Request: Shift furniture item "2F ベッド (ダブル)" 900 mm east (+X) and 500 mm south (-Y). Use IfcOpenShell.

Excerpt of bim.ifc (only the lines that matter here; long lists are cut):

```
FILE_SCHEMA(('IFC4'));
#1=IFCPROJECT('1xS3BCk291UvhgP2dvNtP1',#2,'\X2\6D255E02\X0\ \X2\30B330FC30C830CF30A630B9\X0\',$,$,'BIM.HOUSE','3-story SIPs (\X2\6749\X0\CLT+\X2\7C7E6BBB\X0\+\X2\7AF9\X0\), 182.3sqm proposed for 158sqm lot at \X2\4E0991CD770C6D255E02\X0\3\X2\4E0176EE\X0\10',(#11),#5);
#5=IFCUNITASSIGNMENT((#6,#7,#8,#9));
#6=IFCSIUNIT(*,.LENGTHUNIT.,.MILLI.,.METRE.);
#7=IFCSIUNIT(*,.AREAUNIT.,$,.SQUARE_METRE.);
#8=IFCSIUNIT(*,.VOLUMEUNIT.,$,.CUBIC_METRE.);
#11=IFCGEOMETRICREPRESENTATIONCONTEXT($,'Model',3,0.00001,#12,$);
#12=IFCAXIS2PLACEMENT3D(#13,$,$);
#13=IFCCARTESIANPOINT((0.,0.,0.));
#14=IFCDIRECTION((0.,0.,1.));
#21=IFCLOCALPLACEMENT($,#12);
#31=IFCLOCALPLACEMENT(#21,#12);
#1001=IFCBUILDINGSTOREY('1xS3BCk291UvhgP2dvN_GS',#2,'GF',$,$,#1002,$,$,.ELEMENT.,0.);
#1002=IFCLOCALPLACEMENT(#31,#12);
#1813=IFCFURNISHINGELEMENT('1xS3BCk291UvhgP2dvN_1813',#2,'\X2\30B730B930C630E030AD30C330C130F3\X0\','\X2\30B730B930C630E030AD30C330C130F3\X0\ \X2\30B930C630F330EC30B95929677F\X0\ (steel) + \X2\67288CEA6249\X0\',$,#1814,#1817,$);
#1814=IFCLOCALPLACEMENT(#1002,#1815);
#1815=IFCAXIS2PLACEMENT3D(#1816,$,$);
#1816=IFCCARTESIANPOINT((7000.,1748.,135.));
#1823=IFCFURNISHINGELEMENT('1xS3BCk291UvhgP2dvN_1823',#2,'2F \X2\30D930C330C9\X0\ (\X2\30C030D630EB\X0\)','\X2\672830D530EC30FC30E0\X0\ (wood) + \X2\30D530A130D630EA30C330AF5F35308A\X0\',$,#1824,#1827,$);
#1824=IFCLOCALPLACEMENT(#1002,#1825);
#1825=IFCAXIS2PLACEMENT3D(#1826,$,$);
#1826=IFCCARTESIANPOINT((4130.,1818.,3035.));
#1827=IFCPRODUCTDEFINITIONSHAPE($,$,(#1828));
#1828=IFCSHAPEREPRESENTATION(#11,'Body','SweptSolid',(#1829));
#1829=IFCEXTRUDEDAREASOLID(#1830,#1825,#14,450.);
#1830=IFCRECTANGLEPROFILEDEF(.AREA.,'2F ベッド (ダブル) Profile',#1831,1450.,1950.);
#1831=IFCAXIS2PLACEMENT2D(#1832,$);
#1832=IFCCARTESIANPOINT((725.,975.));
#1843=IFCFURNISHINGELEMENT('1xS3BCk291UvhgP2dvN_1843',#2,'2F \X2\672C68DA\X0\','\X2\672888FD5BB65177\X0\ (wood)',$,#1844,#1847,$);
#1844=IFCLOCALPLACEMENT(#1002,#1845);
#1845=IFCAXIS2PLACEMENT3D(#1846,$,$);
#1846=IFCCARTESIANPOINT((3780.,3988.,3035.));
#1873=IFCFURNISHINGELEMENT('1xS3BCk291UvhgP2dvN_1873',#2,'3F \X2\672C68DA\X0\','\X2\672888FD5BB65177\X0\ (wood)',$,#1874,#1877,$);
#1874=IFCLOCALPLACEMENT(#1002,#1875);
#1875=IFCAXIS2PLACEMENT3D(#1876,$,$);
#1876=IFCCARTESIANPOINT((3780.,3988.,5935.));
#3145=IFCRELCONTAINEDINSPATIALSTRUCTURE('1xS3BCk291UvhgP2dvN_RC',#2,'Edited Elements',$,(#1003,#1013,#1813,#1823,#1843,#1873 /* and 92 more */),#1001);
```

```python
import ifcopenshell
import ifcopenshell.api.geometry
import ifcopenshell.util.placement

model = ifcopenshell.open("bim.ifc")

item = model.by_guid("1xS3BCk291UvhgP2dvN_1823")
matrix = ifcopenshell.util.placement.get_local_placement(item.ObjectPlacement)
matrix[0, 3] += 900.0
matrix[1, 3] -= 500.0
ifcopenshell.api.geometry.edit_object_placement(model, product=item, matrix=matrix, is_si=False)

print(ifcopenshell.util.placement.get_local_placement(item.ObjectPlacement).round(3) + 0.0)

model.write("bim_rev.ifc")
```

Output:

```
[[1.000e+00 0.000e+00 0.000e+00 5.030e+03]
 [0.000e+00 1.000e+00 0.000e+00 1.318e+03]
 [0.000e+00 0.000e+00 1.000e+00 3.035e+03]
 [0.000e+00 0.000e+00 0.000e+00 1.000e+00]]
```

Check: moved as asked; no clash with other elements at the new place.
